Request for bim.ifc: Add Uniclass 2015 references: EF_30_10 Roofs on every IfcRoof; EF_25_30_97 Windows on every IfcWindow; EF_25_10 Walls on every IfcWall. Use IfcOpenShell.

First a look at what the model holds.

```python
import ifcopenshell

model = ifcopenshell.open("bim.ifc")
print(model.schema)
print("classifications:", [c.Name for c in model.by_type("IfcClassification")])
for ifc_class in ("IfcDoor", "IfcRoof", "IfcStair", "IfcWall", "IfcWindow"):
    print(ifc_class, len(model.by_type(ifc_class)))
```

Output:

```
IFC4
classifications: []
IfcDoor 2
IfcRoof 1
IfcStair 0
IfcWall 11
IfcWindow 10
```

```python
import ifcopenshell
import ifcopenshell.api.classification

model = ifcopenshell.open("bim.ifc")

system = ifcopenshell.api.classification.add_classification(model, classification="Uniclass 2015")

codes = {
    "IfcRoof": ("EF_30_10", "Roofs"),
    "IfcWindow": ("EF_25_30_97", "Windows"),
    "IfcWall": ("EF_25_10", "Walls"),
}
for ifc_class, (code, name) in codes.items():
    products = model.by_type(ifc_class)
    ifcopenshell.api.classification.add_reference(
        model, products=products, classification=system, identification=code, name=name
    )
    print(code, len(products))

model.write("bim-out.ifc")
```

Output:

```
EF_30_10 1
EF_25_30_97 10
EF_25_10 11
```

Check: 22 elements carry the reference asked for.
